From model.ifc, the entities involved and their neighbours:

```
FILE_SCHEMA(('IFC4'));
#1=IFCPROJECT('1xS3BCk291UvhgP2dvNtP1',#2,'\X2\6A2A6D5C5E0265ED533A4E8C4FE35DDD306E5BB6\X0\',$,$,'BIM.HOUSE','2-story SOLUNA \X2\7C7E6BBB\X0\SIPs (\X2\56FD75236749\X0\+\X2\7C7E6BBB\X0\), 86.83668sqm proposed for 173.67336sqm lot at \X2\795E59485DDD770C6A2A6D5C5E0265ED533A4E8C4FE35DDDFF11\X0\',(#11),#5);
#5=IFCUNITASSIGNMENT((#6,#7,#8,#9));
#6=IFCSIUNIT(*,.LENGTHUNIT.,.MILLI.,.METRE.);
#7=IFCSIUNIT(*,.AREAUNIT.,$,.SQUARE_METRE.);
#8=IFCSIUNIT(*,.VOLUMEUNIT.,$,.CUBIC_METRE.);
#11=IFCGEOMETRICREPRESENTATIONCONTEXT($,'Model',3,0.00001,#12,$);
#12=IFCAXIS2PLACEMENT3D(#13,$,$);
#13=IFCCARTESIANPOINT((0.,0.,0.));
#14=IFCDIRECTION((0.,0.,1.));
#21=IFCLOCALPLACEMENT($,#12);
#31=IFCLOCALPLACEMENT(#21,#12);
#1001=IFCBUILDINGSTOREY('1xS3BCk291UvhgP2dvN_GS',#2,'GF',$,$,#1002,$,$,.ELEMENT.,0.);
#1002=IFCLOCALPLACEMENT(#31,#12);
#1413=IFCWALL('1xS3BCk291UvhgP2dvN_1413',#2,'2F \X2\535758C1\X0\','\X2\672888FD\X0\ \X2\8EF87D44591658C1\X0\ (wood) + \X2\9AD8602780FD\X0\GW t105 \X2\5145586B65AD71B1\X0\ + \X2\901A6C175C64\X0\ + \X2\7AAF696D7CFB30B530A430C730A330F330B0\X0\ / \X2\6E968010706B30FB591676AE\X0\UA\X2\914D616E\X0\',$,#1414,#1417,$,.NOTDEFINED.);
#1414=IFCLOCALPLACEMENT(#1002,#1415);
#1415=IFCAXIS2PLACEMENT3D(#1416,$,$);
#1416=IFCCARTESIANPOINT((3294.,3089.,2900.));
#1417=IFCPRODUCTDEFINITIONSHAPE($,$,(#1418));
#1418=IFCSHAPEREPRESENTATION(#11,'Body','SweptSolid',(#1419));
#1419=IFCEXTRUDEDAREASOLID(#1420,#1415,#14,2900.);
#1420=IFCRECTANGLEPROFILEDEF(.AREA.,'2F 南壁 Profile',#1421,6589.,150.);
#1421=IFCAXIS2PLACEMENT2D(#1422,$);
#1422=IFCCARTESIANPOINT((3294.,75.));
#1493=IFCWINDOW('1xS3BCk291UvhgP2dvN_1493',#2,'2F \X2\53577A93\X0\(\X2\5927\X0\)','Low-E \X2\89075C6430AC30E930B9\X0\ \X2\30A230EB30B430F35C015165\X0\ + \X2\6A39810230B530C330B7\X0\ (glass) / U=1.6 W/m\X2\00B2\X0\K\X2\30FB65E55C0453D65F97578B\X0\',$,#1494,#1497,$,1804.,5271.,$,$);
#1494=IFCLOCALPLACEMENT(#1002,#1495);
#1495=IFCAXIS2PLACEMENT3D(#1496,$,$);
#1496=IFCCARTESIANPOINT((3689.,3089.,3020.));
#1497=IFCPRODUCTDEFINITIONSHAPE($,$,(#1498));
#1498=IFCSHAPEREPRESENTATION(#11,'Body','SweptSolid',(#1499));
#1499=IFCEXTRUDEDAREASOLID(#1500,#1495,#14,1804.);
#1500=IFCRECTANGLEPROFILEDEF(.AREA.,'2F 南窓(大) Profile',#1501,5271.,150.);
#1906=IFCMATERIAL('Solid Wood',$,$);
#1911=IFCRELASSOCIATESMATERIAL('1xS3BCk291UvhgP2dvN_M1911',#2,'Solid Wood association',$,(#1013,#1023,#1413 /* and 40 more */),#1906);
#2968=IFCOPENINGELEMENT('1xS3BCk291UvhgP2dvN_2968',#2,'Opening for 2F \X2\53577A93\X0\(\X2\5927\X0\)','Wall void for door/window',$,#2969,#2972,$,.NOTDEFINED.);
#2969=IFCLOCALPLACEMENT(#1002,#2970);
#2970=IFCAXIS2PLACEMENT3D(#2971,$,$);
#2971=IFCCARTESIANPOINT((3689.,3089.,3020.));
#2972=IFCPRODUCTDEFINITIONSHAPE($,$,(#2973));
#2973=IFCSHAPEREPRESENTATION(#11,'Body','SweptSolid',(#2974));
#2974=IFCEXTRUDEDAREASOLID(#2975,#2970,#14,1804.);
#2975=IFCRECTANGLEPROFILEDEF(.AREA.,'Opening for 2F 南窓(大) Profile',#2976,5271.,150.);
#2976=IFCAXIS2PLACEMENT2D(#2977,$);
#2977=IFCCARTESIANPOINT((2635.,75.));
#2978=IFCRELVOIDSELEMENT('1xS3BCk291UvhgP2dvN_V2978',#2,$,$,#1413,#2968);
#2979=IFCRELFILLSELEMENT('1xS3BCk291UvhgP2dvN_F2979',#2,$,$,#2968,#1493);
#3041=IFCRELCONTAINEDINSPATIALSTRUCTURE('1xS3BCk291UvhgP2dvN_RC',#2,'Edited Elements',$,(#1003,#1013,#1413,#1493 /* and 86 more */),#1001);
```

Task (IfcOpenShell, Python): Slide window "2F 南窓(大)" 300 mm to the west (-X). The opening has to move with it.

```python
import ifcopenshell
import ifcopenshell.api.geometry
import ifcopenshell.util.placement
import ifcopenshell.util.unit

model = ifcopenshell.open("model.ifc")
unit_scale = ifcopenshell.util.unit.calculate_unit_scale(model)

window = model.by_id(1493)
opening = window.FillsVoids[0].RelatingOpeningElement
wall = opening.VoidsElements[0].RelatingBuildingElement

wall_matrix = ifcopenshell.util.placement.get_local_placement(wall.ObjectPlacement)
shift = wall_matrix[:3, 0] * -0.3 / unit_scale
before = ifcopenshell.util.placement.get_local_placement(window.ObjectPlacement)[:3, 3].copy()

# The window is not placed relative to its opening, so move both.
for product in (opening, window):
    matrix = ifcopenshell.util.placement.get_local_placement(product.ObjectPlacement)
    matrix[:3, 3] += shift
    ifcopenshell.api.geometry.edit_object_placement(model, product=product, matrix=matrix, is_si=False)

after = ifcopenshell.util.placement.get_local_placement(window.ObjectPlacement)[:3, 3]
print("window moved by", (after - before).round(3) + 0.0)

model.write("model_updated.ifc")
```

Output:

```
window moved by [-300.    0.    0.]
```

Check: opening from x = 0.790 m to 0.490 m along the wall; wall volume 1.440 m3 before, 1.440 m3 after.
